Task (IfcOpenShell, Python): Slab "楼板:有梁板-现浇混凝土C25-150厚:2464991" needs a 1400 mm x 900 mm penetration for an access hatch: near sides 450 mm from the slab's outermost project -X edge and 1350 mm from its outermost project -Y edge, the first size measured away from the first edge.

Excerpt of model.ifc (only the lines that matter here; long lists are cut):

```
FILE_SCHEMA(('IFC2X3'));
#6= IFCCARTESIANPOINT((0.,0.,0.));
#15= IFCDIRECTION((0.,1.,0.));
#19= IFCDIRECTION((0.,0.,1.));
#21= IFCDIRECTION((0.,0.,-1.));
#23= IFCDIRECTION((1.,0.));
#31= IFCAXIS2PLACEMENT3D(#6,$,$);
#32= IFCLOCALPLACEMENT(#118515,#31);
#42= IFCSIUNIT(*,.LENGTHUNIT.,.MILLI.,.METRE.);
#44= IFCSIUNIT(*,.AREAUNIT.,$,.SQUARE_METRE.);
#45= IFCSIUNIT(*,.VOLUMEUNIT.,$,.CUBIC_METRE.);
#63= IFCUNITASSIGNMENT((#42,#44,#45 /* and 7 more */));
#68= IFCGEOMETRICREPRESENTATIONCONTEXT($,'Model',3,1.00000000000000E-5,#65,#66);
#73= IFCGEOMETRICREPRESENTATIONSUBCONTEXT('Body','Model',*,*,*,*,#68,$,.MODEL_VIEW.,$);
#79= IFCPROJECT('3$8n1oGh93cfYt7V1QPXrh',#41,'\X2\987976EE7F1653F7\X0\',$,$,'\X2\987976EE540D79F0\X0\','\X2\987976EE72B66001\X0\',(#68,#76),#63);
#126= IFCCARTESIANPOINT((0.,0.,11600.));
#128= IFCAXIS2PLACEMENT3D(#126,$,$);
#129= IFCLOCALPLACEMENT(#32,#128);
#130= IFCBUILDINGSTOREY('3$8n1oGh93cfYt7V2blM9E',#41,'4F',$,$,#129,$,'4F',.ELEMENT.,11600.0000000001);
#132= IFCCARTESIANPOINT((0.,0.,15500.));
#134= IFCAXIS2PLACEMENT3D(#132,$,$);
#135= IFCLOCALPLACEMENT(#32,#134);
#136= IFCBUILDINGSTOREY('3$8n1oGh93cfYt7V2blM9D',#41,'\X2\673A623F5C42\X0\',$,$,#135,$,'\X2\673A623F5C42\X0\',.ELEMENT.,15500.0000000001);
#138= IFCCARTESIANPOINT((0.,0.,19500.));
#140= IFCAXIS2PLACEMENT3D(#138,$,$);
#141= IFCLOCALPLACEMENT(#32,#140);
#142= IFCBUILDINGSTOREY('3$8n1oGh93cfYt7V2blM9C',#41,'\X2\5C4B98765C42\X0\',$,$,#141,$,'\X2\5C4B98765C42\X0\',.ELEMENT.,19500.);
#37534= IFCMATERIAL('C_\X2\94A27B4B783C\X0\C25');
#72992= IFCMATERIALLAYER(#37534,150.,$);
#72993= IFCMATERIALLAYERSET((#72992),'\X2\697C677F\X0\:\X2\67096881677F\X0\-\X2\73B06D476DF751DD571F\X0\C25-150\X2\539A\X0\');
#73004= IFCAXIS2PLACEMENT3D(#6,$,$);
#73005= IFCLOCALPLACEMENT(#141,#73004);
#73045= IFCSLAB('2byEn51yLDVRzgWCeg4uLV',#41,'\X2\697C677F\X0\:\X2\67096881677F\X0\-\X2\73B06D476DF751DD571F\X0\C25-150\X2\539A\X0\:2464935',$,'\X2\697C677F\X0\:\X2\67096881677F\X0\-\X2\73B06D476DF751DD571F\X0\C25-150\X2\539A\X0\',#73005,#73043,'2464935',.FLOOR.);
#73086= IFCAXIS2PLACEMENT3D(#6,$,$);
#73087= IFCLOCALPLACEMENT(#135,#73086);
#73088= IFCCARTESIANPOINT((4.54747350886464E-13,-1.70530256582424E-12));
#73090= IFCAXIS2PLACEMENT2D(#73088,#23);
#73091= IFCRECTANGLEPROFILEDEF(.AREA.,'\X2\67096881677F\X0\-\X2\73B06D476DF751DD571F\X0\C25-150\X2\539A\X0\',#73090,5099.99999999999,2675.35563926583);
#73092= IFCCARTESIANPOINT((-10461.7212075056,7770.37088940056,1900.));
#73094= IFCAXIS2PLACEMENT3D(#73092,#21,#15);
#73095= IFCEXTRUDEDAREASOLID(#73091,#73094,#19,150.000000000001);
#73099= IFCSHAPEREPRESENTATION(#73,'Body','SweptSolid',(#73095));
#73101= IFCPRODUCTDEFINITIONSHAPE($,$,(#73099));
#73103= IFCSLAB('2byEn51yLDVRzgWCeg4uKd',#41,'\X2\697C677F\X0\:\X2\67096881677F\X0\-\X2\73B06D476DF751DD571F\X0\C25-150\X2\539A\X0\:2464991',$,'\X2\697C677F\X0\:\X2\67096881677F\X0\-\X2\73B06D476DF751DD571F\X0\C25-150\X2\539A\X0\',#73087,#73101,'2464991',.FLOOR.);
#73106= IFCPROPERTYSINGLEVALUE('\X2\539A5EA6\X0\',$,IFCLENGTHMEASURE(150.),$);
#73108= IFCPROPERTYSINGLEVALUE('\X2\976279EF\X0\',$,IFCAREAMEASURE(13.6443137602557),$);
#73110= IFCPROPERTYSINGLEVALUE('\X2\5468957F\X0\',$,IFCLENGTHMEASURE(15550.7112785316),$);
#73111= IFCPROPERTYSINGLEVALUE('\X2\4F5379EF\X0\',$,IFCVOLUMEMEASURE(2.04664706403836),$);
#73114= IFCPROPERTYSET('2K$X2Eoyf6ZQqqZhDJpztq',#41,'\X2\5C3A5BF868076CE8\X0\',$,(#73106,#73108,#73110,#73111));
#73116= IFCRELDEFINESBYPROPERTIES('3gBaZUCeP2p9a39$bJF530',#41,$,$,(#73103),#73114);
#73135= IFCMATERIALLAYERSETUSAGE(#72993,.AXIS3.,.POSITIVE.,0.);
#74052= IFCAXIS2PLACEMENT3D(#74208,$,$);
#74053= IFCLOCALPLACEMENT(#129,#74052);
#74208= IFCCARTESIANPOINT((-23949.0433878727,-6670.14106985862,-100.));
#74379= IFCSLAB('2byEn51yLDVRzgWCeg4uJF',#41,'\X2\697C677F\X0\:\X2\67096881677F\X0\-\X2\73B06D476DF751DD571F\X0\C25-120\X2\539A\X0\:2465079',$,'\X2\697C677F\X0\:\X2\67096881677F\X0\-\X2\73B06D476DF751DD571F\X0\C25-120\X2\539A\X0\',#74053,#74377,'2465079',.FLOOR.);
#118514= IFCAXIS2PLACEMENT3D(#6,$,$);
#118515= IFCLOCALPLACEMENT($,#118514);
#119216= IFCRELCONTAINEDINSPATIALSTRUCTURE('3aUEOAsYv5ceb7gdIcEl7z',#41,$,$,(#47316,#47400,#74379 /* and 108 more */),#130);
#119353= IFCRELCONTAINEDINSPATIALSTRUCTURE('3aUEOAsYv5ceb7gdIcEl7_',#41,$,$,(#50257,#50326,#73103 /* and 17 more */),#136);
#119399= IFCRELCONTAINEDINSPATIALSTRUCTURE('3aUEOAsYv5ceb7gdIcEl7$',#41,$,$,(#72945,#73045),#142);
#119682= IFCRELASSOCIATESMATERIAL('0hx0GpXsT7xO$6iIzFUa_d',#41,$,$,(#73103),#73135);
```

```python
import numpy as np
import ifcopenshell
import ifcopenshell.api.feature
import ifcopenshell.api.geometry
import ifcopenshell.api.pset
import ifcopenshell.api.root
import ifcopenshell.geom
import ifcopenshell.util.element
import ifcopenshell.util.placement
import ifcopenshell.util.representation
import ifcopenshell.util.shape
import ifcopenshell.util.unit

model = ifcopenshell.open("model.ifc")
unit_scale = ifcopenshell.util.unit.calculate_unit_scale(model)
area_scale = ifcopenshell.util.unit.calculate_unit_scale(model, "AREAUNIT")
volume_scale = ifcopenshell.util.unit.calculate_unit_scale(model, "VOLUMEUNIT")
settings = ifcopenshell.geom.settings()


def volume(element):
    """Net volume in cubic metres, openings subtracted."""
    shape = ifcopenshell.geom.create_shape(settings, element)
    return ifcopenshell.util.shape.get_volume(shape.geometry)


slab = model.by_guid("2byEn51yLDVRzgWCeg4uKd")
before = volume(slab)

# Extent in the slab's own axes, in metres. The edges named are its -X and -Y sides.
slab_shape = ifcopenshell.geom.create_shape(settings, slab)
vertices = ifcopenshell.util.shape.get_vertices(slab_shape.geometry)
x_min, y_min, bottom = vertices.min(axis=0)
top = vertices[:, 2].max()

opening = ifcopenshell.api.root.create_entity(model, ifc_class="IfcOpeningElement", name="Access hatch opening")
context = ifcopenshell.util.representation.get_context(model, "Model", "Body", "MODEL_VIEW")
width, depth = 1.4, 0.9
outline = [(0.0, 0.0), (width, 0.0), (width, depth), (0.0, depth), (0.0, 0.0)]
# Overshoot both faces by 50 mm so the cut is clean.
shape = ifcopenshell.api.geometry.add_slab_representation(
    model, context=context, depth=top - bottom + 0.1, polyline=outline
)
ifcopenshell.api.geometry.assign_representation(model, product=opening, representation=shape)

matrix = ifcopenshell.util.placement.get_local_placement(slab.ObjectPlacement)
matrix[:, 3] = matrix @ np.append(np.array([x_min + 0.45, y_min + 1.35, bottom - 0.05]) / unit_scale, 1.0)
ifcopenshell.api.geometry.edit_object_placement(model, product=opening, matrix=matrix, is_si=False)
ifcopenshell.api.feature.add_feature(model, feature=opening, element=slab)

after = volume(slab)

# Update the slab's stored quantities.
pset = model.by_id(ifcopenshell.util.element.get_pset(slab, "尺寸标注", should_inherit=False)["id"])
ifcopenshell.api.pset.edit_pset(model, pset=pset, properties={
    "面积": model.create_entity("IfcAreaMeasure", after / (top - bottom) / area_scale),
    "体积": model.create_entity("IfcVolumeMeasure", after / volume_scale),
})

print(f"slab volume {before:.3f} -> {after:.3f} m3")

model.write("model-out.ifc")
```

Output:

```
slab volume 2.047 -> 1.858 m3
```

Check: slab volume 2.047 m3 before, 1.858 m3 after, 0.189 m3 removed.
